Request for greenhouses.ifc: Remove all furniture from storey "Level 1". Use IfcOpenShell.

First a look at what the model holds.

```python
import ifcopenshell
import ifcopenshell.util.element

model = ifcopenshell.open("greenhouses.ifc")
print(model.schema)
storey = next(s for s in model.by_type("IfcBuildingStorey") if s.Name == "Level 1")
furniture = [e for e in ifcopenshell.util.element.get_decomposition(storey) if e.is_a("IfcFurnishingElement")]
seen = {}
for e in furniture:
    element_type = ifcopenshell.util.element.get_type(e)
    name = element_type.Name if element_type not in (None, e) else None
    seen[name] = seen.get(name, 0) + 1
for name, count in sorted(seen.items(), key=str):
    print(count, "x", name)
```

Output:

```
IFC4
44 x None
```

```python
import ifcopenshell
import ifcopenshell.api.root
import ifcopenshell.util.element

model = ifcopenshell.open("greenhouses.ifc")

storey = next(s for s in model.by_type("IfcBuildingStorey") if s.Name == "Level 1")
furniture = [e for e in ifcopenshell.util.element.get_decomposition(storey) if e.is_a("IfcFurnishingElement")]

for e in furniture:
    ifcopenshell.api.root.remove_product(model, product=e)
print(len(furniture), "removed")

model.write("greenhouses-out.ifc")
```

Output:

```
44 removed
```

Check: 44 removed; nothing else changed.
